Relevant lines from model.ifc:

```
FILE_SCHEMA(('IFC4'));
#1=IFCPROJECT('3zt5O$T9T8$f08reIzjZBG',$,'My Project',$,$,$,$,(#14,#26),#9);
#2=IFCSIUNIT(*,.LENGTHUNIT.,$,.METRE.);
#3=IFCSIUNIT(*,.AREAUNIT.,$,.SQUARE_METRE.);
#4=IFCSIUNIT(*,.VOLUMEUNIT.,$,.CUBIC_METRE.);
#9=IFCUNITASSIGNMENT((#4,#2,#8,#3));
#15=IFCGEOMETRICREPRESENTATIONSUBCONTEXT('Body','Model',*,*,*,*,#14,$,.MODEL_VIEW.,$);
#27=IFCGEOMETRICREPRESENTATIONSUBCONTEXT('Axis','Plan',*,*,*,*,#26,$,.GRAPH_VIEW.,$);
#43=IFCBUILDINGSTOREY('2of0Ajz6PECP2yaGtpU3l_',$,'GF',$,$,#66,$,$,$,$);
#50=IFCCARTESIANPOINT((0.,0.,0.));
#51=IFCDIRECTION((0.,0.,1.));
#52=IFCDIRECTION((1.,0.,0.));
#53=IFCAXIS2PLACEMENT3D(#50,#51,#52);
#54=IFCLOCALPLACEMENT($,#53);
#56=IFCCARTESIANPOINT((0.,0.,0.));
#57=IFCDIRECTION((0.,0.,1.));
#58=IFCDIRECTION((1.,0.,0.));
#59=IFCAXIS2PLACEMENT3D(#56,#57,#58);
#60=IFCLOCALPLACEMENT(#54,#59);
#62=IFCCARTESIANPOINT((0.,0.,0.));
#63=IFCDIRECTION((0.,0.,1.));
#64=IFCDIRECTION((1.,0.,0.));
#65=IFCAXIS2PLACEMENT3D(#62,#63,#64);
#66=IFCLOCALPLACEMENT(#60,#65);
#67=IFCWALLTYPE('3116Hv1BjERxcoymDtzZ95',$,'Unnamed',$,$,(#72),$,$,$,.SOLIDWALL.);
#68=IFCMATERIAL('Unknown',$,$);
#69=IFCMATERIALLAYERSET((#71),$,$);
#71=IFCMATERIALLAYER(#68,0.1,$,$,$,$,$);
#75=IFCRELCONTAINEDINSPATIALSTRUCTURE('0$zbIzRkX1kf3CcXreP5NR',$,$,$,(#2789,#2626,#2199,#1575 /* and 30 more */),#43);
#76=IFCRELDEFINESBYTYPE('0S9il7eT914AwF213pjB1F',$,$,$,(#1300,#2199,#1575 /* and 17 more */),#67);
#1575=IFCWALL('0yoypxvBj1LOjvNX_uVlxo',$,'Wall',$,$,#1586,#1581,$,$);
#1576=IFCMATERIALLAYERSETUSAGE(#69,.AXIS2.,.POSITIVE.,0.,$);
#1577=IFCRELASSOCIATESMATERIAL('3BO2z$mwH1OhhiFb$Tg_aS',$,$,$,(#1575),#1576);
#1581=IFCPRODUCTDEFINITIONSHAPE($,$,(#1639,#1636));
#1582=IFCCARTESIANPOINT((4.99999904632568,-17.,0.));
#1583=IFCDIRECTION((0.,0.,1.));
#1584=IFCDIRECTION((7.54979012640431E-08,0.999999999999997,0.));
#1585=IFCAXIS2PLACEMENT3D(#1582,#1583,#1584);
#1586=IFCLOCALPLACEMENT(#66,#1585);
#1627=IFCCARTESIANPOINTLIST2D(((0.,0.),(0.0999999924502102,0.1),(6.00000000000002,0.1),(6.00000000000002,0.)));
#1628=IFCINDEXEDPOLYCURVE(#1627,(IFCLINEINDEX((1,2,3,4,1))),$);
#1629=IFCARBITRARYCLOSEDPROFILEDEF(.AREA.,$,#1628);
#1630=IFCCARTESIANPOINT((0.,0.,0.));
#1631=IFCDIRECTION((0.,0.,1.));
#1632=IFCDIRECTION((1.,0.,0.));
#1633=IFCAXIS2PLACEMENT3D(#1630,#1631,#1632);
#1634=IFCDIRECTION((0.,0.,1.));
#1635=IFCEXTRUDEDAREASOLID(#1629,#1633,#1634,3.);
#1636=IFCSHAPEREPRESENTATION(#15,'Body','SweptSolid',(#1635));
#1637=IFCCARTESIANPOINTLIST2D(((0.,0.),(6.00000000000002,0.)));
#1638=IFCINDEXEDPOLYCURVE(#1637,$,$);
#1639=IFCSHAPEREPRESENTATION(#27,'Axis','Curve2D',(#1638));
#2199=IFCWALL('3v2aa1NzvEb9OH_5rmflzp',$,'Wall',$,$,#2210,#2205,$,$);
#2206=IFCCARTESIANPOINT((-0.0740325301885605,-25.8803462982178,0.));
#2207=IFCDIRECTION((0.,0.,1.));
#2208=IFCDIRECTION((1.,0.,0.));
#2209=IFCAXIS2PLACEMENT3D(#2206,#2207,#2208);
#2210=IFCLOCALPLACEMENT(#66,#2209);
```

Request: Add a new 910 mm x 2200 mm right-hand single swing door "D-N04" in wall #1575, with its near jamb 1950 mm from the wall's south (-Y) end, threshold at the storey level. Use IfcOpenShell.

```python
import numpy as np
import ifcopenshell
import ifcopenshell.api.feature
import ifcopenshell.api.geometry
import ifcopenshell.api.root
import ifcopenshell.api.spatial
import ifcopenshell.geom
import ifcopenshell.util.element
import ifcopenshell.util.placement
import ifcopenshell.util.representation
import ifcopenshell.util.shape
import ifcopenshell.util.unit

model = ifcopenshell.open("model.ifc")
unit_scale = ifcopenshell.util.unit.calculate_unit_scale(model)
settings = ifcopenshell.geom.settings()


def volume(element):
    """Net volume in cubic metres, openings subtracted."""
    shape = ifcopenshell.geom.create_shape(settings, element)
    return ifcopenshell.util.shape.get_volume(shape.geometry)


wall = model.by_guid("0yoypxvBj1LOjvNX_uVlxo")
storey = ifcopenshell.util.element.get_container(wall, ifc_class="IfcBuildingStorey")
context = ifcopenshell.util.representation.get_context(model, "Model", "Body", "MODEL_VIEW")
before = volume(wall)

width, height, from_end, sill = 0.91, 2.2, 1.95, 0.0  # metres

# The wall runs along its own X axis, and the end named is its -X end.
wall_shape = ifcopenshell.geom.create_shape(settings, wall)
x, y, z = ifcopenshell.util.shape.get_vertices(wall_shape.geometry).T
start = x.min() + from_end
face, thickness = float(y.min()), float(y.max() - y.min())
wall_matrix = ifcopenshell.util.placement.get_local_placement(wall.ObjectPlacement)
level = ifcopenshell.util.placement.get_local_placement(storey.ObjectPlacement)[2, 3]


def in_wall(x, y):
    """Placement at x, y metres in the wall's axes, at sill height."""
    matrix = wall_matrix.copy()
    matrix[:, 3] = wall_matrix @ np.array([x / unit_scale, y / unit_scale, 0.0, 1.0])
    matrix[2, 3] = level + sill / unit_scale
    return matrix


# Opening: a box that overshoots both wall faces by 50 mm.
opening = ifcopenshell.api.root.create_entity(model, ifc_class="IfcOpeningElement", predefined_type="OPENING")
box = ifcopenshell.api.geometry.add_wall_representation(
    model, context=context, length=width, height=height, thickness=thickness + 0.1
)
ifcopenshell.api.geometry.assign_representation(model, product=opening, representation=box)
ifcopenshell.api.geometry.edit_object_placement(model, product=opening, matrix=in_wall(start, face - 0.05), is_si=False)
ifcopenshell.api.feature.add_feature(model, feature=opening, element=wall)

door = ifcopenshell.api.root.create_entity(model, ifc_class="IfcDoor", name="D-N04", predefined_type="DOOR")
door.OverallWidth, door.OverallHeight = width / unit_scale, height / unit_scale
door.OperationType = "SINGLE_SWING_RIGHT"
body = ifcopenshell.api.geometry.add_door_representation(
    model,
    context=context,
    overall_width=door.OverallWidth,
    overall_height=door.OverallHeight,
    operation_type="SINGLE_SWING_RIGHT",
    lining_properties={"LiningDepth": thickness / unit_scale, "ThresholdDepth": thickness / unit_scale},
)
ifcopenshell.api.geometry.assign_representation(model, product=door, representation=body)
ifcopenshell.api.spatial.assign_container(model, products=[door], relating_structure=storey)
ifcopenshell.api.feature.add_filling(model, opening=opening, element=door)

# The lining spans the wall, so the door starts at the wall face.
ifcopenshell.api.geometry.edit_object_placement(model, product=door, matrix=in_wall(start, face), is_si=False)

after = volume(wall)

print(f"wall volume {before:.3f} -> {after:.3f} m3")

model.write("model_rev.ifc")
```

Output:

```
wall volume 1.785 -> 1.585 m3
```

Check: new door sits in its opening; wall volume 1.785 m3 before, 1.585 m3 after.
